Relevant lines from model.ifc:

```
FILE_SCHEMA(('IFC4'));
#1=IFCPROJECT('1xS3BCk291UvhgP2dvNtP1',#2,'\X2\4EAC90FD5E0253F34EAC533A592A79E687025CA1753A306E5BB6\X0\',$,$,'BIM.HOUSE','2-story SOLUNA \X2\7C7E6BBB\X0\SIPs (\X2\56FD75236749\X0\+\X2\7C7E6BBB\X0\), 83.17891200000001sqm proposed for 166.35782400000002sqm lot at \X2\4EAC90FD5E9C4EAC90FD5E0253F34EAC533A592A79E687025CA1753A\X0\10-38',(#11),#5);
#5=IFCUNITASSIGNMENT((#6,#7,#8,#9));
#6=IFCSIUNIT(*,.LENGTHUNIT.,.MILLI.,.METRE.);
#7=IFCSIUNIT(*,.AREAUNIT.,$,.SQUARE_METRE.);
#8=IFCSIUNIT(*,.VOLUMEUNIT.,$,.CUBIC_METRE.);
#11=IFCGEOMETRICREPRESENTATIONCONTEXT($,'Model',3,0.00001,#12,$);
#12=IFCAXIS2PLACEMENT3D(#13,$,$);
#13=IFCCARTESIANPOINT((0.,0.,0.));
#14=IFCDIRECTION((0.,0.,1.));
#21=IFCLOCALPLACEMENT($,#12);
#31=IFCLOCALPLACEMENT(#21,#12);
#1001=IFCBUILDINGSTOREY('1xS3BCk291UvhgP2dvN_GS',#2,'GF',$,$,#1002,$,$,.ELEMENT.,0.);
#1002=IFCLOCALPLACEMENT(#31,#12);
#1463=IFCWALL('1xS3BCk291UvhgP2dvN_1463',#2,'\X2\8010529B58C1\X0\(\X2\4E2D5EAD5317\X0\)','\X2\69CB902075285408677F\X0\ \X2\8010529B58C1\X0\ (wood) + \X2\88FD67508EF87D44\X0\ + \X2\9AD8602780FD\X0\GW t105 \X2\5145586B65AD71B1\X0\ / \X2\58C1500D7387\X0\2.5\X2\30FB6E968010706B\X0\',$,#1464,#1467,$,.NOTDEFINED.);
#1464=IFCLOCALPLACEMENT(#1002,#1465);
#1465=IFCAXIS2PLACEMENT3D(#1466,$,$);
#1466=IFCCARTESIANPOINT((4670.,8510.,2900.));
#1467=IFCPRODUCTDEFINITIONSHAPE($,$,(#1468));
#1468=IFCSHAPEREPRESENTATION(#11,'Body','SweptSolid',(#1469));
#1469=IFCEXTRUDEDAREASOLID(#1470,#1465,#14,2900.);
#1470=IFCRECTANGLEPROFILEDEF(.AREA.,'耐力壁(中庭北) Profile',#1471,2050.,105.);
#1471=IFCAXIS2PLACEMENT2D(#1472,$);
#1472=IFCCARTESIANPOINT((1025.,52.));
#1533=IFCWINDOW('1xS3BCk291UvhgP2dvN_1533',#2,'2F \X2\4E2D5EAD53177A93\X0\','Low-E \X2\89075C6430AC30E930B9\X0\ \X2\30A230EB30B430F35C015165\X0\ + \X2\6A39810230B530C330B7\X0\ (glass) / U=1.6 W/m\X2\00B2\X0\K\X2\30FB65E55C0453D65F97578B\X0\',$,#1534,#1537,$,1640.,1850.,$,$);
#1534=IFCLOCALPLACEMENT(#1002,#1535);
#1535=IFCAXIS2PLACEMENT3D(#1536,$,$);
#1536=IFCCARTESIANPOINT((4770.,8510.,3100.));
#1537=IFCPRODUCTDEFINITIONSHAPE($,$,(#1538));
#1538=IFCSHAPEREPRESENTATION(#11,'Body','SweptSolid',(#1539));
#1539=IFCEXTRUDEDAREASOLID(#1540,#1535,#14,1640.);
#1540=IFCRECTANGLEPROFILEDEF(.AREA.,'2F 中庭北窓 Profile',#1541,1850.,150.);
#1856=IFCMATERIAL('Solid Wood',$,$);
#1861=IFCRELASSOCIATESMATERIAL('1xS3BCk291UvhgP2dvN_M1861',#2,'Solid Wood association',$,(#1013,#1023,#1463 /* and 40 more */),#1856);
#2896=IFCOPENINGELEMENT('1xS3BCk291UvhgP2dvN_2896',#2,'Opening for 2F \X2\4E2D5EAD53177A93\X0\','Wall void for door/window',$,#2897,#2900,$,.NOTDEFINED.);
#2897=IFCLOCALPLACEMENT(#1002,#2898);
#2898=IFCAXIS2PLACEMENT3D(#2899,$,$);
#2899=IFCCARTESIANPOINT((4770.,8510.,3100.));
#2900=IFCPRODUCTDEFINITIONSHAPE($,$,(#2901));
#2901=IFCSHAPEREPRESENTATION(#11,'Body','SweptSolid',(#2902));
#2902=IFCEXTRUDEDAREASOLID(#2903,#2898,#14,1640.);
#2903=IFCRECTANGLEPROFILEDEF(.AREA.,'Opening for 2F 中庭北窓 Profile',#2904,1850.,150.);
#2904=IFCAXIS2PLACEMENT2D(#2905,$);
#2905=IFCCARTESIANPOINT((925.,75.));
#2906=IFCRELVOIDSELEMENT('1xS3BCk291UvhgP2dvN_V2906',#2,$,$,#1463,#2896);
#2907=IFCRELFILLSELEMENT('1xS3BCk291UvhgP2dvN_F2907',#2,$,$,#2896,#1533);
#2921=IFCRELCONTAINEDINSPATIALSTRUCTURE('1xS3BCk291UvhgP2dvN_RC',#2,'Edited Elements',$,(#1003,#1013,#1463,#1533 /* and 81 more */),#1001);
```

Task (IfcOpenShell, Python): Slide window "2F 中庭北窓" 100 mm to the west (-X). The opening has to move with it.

```python
import ifcopenshell
import ifcopenshell.api.geometry
import ifcopenshell.util.placement

model = ifcopenshell.open("model.ifc")

window = model.by_id(1533)
opening = window.FillsVoids[0].RelatingOpeningElement
wall = opening.VoidsElements[0].RelatingBuildingElement

wall_matrix = ifcopenshell.util.placement.get_local_placement(wall.ObjectPlacement)
shift = wall_matrix[:3, 0] * -100.0
before = ifcopenshell.util.placement.get_local_placement(window.ObjectPlacement)[:3, 3].copy()

# The window is not placed relative to its opening, so move both.
for product in (opening, window):
    matrix = ifcopenshell.util.placement.get_local_placement(product.ObjectPlacement)
    matrix[:3, 3] += shift
    ifcopenshell.api.geometry.edit_object_placement(model, product=product, matrix=matrix, is_si=False)

after = ifcopenshell.util.placement.get_local_placement(window.ObjectPlacement)[:3, 3]
print("window moved by", (after - before).round(3) + 0.0)

model.write("model_v2.ifc")
```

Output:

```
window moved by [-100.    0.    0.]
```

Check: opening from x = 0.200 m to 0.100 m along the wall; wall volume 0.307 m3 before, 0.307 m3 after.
